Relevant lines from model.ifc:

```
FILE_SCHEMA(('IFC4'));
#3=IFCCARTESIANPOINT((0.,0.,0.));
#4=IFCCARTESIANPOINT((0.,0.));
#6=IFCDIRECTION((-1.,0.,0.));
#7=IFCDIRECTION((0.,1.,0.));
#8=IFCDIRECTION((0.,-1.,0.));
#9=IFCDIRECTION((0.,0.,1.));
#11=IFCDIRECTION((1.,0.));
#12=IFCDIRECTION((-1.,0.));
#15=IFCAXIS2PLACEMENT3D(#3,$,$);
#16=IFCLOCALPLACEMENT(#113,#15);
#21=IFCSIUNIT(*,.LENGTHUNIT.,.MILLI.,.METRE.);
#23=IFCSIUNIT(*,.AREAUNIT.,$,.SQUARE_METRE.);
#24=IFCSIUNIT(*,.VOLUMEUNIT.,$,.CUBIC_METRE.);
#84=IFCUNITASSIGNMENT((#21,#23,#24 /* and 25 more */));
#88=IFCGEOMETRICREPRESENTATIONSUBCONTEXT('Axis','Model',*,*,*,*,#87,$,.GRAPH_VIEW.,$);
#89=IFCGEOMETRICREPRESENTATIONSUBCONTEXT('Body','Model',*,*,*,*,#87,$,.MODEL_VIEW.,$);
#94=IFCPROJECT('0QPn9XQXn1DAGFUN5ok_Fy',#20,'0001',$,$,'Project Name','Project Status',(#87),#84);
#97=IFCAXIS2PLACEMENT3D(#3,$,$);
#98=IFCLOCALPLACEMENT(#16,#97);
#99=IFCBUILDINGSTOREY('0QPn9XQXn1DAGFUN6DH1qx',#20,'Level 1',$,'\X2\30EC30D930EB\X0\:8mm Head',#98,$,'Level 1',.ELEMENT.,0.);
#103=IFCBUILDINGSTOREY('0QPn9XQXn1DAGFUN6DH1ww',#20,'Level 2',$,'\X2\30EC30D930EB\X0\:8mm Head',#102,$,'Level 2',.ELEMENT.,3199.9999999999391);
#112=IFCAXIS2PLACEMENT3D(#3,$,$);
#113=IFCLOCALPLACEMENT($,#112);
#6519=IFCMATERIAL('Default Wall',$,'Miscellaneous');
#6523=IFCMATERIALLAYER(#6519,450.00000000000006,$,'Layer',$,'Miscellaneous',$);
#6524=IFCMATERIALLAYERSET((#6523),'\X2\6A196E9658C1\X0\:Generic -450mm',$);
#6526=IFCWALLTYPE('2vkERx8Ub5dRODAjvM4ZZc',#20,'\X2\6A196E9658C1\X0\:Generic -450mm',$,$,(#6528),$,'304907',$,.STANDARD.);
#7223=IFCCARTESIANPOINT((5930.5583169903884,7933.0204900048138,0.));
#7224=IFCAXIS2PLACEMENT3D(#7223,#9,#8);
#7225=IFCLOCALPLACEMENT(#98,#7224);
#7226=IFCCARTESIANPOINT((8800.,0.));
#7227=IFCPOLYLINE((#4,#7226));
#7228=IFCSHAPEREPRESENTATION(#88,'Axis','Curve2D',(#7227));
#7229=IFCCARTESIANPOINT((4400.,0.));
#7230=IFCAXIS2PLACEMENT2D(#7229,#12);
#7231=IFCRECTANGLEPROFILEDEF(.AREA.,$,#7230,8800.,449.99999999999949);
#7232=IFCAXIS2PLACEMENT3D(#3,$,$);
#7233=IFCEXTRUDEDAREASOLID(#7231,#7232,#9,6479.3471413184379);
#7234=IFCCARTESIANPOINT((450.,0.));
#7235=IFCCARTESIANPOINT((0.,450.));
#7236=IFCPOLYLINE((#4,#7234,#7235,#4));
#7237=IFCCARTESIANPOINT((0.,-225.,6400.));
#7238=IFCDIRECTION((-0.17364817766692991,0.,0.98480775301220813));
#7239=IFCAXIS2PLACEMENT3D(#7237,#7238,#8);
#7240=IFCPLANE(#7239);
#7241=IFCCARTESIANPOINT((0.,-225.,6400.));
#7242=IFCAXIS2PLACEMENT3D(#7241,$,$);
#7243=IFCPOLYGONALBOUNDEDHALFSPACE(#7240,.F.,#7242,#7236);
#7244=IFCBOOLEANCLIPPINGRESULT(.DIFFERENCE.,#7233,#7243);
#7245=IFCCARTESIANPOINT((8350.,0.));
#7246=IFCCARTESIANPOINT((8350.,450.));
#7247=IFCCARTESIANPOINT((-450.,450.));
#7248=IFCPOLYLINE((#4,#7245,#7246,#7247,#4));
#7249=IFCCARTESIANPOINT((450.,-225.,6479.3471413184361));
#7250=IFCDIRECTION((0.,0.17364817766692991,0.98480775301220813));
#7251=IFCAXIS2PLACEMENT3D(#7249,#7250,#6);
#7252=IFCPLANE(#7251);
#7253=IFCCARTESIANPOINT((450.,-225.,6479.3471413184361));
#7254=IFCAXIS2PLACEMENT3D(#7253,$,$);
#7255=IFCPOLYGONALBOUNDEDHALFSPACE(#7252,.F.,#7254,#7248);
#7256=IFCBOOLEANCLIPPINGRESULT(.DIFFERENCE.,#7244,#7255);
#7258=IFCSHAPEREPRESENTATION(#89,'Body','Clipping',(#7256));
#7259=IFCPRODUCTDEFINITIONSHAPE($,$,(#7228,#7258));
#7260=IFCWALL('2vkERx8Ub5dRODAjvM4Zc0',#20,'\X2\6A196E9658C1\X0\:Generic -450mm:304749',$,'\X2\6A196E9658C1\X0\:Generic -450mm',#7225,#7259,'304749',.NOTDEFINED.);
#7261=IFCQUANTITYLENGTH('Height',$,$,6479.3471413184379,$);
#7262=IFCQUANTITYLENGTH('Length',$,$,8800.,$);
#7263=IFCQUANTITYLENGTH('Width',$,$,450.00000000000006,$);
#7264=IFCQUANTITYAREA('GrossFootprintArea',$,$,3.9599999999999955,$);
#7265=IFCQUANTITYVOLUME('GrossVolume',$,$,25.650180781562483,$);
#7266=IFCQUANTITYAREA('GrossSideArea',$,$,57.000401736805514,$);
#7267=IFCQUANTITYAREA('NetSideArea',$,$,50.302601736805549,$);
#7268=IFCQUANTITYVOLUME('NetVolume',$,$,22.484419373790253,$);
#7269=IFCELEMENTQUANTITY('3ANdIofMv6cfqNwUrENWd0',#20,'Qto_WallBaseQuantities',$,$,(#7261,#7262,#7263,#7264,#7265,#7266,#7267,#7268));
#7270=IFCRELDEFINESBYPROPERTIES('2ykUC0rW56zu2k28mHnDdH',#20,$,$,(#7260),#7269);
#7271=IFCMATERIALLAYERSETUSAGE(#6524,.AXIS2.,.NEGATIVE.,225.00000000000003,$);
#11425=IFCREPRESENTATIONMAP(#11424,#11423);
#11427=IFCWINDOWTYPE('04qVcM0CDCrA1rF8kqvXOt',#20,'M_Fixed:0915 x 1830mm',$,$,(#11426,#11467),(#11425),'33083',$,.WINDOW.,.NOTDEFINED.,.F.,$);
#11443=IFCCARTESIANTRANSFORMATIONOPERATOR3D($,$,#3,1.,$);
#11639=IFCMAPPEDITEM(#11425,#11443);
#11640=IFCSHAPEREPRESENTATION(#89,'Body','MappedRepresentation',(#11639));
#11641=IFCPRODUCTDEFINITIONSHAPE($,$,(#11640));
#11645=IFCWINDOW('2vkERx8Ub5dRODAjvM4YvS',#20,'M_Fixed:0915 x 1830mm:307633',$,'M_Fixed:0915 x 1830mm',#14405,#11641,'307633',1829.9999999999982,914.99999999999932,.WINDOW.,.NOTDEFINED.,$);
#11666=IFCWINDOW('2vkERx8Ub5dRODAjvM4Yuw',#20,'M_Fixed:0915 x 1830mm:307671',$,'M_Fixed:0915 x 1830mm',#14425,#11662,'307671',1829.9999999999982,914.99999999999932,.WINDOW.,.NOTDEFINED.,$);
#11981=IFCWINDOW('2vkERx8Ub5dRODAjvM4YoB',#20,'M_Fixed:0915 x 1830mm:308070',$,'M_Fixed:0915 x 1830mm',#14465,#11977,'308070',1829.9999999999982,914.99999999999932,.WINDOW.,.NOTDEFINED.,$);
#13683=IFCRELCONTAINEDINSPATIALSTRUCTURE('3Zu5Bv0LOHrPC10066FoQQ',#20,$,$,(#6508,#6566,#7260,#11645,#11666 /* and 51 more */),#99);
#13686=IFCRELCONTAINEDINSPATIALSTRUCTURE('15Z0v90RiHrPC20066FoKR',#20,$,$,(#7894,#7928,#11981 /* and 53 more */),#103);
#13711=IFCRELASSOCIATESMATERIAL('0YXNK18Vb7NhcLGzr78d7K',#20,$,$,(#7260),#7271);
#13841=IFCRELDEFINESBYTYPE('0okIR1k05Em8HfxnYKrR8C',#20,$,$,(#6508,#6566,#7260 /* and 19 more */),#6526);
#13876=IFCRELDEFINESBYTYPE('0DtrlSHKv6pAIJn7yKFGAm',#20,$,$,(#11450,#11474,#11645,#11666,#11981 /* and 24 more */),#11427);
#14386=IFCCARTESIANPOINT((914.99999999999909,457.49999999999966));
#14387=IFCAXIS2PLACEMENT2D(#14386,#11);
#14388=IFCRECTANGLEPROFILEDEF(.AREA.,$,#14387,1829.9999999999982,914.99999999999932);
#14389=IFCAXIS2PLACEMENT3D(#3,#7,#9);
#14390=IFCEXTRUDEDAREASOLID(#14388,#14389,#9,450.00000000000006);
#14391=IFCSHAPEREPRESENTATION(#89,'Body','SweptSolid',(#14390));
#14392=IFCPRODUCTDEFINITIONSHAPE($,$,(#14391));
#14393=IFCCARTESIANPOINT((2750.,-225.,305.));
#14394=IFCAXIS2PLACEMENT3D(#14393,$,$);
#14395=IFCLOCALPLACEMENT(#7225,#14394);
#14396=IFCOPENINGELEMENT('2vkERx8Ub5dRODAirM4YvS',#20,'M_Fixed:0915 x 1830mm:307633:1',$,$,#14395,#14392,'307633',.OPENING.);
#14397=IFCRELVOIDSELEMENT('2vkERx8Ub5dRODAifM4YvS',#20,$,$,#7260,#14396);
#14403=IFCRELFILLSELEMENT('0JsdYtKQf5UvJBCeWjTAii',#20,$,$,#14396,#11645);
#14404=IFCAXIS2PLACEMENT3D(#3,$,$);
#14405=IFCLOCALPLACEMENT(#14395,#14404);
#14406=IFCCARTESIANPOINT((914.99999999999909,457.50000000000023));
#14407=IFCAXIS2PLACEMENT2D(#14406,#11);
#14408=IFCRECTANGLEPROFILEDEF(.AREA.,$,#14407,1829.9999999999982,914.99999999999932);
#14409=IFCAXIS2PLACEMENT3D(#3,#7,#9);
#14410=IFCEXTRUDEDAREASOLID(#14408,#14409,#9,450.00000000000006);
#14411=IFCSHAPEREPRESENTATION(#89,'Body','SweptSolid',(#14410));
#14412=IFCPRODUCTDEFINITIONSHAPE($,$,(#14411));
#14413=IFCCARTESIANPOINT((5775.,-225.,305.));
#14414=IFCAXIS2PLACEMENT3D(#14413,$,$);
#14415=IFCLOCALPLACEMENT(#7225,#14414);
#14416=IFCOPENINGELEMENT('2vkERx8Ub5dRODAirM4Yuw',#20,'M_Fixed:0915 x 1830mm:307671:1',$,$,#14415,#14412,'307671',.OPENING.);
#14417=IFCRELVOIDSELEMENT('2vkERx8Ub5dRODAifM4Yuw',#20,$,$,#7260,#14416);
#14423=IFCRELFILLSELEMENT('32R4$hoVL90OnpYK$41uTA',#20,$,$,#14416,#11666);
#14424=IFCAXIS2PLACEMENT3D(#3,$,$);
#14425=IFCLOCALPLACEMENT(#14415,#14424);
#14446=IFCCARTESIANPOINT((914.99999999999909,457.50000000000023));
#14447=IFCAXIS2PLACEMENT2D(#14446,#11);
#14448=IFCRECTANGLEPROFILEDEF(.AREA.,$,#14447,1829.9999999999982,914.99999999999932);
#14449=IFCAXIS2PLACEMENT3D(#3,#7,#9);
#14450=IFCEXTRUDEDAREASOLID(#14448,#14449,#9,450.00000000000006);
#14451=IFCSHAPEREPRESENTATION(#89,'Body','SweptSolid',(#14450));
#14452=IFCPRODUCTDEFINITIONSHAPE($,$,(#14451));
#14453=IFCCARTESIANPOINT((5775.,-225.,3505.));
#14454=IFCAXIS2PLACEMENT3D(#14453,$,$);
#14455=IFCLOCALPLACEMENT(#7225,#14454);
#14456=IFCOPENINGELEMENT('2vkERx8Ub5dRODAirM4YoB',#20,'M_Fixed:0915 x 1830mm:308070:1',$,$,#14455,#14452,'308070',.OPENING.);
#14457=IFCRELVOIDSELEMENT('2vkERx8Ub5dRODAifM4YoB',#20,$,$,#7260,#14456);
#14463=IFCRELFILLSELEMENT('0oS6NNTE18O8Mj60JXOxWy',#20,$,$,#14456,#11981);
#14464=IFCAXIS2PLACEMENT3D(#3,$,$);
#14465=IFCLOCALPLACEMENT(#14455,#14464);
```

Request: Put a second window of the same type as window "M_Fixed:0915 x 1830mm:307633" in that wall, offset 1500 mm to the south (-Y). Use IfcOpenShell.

```python
import ifcopenshell
import ifcopenshell.api.feature
import ifcopenshell.api.geometry
import ifcopenshell.api.pset
import ifcopenshell.api.root
import ifcopenshell.geom
import ifcopenshell.util.element
import ifcopenshell.util.placement
import ifcopenshell.util.shape
import ifcopenshell.util.unit

model = ifcopenshell.open("model.ifc")
unit_scale = ifcopenshell.util.unit.calculate_unit_scale(model)
area_scale = ifcopenshell.util.unit.calculate_unit_scale(model, "AREAUNIT")
volume_scale = ifcopenshell.util.unit.calculate_unit_scale(model, "VOLUMEUNIT")
settings = ifcopenshell.geom.settings()


def volume(element):
    """Net volume in cubic metres, openings subtracted."""
    shape = ifcopenshell.geom.create_shape(settings, element)
    return ifcopenshell.util.shape.get_volume(shape.geometry)


def reuse_history(source, copy):
    """copy_class also copies each property set's owner history, people and application; keep the originals."""
    for rel in copy.IsDefinedBy:
        if rel.is_a("IfcRelDefinesByProperties") and (history := rel.RelatingPropertyDefinition.OwnerHistory):
            rel.RelatingPropertyDefinition.OwnerHistory = source.OwnerHistory
            ifcopenshell.util.element.remove_deep2(model, history)


window = model.by_guid("2vkERx8Ub5dRODAjvM4YvS")
opening = window.FillsVoids[0].RelatingOpeningElement
wall = opening.VoidsElements[0].RelatingBuildingElement
before = volume(wall)
shift = ifcopenshell.util.placement.get_local_placement(wall.ObjectPlacement)[:3, 0] * 1.5 / unit_scale

# copy_class copies the void relationship, type, container and properties, but no geometry.
new_opening = ifcopenshell.api.root.copy_class(model, product=opening)
new_opening.Representation = ifcopenshell.util.element.copy_deep(
    model, opening.Representation, exclude=["IfcGeometricRepresentationContext", "IfcRepresentationMap"]
)
new_opening.Name = "M_Fixed:0915 x 1830mm"
new_opening.Tag = None
reuse_history(opening, new_opening)
new_window = ifcopenshell.api.root.copy_class(model, product=window)
new_window.Representation = ifcopenshell.util.element.copy_deep(
    model, window.Representation, exclude=["IfcGeometricRepresentationContext", "IfcRepresentationMap"]
)
new_window.Name = "M_Fixed:0915 x 1830mm"
new_window.Tag = None
reuse_history(window, new_window)
ifcopenshell.api.feature.add_filling(model, opening=new_opening, element=new_window)

for old, new in ((opening, new_opening), (window, new_window)):
    matrix = ifcopenshell.util.placement.get_local_placement(old.ObjectPlacement)
    matrix[:3, 3] += shift
    ifcopenshell.api.geometry.edit_object_placement(model, product=new, matrix=matrix, is_si=False)

after = volume(wall)
thickness = 0.45  # wall thickness in metres

# Update the wall's stored quantities.
qto = model.by_id(ifcopenshell.util.element.get_pset(wall, "Qto_WallBaseQuantities", should_inherit=False)["id"])
ifcopenshell.api.pset.edit_qto(model, qto=qto, properties={
    "NetSideArea": after / thickness / area_scale,
    "NetVolume": after / volume_scale,
})

print(f"wall volume {before:.3f} -> {after:.3f} m3")

model.write("model_rev.ifc")
```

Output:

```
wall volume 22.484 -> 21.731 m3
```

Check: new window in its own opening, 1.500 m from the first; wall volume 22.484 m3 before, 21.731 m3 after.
